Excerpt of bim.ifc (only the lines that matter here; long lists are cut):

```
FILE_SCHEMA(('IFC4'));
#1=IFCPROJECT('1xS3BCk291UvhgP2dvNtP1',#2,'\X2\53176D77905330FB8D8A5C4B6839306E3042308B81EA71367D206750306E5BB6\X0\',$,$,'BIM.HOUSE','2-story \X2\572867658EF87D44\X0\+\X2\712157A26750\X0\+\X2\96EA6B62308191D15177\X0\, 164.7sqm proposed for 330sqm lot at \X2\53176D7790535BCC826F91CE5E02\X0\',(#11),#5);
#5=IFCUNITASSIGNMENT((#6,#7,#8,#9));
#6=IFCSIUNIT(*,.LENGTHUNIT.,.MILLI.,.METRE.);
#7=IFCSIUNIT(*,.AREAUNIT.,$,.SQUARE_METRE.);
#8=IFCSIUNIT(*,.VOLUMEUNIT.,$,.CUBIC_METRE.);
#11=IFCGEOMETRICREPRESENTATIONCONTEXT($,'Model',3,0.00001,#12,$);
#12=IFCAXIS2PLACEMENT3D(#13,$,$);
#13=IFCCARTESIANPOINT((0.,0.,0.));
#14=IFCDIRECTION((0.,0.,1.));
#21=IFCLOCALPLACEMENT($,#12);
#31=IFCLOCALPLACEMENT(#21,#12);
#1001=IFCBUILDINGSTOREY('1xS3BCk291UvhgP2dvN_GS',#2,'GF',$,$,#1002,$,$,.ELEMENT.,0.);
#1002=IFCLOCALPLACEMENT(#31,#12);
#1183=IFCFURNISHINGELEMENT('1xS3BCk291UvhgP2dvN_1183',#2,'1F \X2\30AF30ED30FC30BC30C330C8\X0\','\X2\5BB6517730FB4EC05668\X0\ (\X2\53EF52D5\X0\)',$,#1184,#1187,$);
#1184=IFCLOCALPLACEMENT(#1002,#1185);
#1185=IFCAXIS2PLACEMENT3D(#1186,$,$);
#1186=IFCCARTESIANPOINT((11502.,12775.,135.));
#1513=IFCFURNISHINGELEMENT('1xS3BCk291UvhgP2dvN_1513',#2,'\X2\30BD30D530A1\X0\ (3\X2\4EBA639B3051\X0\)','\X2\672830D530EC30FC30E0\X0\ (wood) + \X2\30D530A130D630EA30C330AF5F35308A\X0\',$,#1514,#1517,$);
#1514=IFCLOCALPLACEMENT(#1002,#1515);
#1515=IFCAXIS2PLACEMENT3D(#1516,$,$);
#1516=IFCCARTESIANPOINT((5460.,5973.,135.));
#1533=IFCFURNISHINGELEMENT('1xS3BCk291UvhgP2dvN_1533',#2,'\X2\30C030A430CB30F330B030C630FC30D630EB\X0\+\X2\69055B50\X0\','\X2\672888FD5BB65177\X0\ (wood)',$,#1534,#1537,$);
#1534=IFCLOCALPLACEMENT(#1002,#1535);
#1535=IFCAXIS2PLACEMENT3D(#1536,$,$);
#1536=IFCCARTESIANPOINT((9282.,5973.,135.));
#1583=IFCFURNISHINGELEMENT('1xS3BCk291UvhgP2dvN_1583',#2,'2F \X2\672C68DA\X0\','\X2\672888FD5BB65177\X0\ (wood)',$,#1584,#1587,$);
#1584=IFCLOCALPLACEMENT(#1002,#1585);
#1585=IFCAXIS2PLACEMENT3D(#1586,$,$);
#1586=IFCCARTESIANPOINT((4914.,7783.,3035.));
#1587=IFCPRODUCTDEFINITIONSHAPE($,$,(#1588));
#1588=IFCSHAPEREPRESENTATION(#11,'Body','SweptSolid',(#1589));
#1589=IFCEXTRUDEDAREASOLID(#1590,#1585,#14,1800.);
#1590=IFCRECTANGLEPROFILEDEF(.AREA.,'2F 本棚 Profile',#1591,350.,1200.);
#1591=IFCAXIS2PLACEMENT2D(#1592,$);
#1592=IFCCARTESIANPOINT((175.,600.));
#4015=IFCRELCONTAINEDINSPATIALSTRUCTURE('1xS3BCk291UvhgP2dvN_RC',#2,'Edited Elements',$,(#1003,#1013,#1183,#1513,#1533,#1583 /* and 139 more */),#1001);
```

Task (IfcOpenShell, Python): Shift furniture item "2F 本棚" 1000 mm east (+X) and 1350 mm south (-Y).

```python
import ifcopenshell
import ifcopenshell.api.geometry
import ifcopenshell.util.placement

model = ifcopenshell.open("bim.ifc")

item = model.by_guid("1xS3BCk291UvhgP2dvN_1583")
matrix = ifcopenshell.util.placement.get_local_placement(item.ObjectPlacement)
matrix[0, 3] += 1000.0
matrix[1, 3] -= 1350.0
ifcopenshell.api.geometry.edit_object_placement(model, product=item, matrix=matrix, is_si=False)

print(ifcopenshell.util.placement.get_local_placement(item.ObjectPlacement).round(3) + 0.0)

model.write("bim_updated.ifc")
```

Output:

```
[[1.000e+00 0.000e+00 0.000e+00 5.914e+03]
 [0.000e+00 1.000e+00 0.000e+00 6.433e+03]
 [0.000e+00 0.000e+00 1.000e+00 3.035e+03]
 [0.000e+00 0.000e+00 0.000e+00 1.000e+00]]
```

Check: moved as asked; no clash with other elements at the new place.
